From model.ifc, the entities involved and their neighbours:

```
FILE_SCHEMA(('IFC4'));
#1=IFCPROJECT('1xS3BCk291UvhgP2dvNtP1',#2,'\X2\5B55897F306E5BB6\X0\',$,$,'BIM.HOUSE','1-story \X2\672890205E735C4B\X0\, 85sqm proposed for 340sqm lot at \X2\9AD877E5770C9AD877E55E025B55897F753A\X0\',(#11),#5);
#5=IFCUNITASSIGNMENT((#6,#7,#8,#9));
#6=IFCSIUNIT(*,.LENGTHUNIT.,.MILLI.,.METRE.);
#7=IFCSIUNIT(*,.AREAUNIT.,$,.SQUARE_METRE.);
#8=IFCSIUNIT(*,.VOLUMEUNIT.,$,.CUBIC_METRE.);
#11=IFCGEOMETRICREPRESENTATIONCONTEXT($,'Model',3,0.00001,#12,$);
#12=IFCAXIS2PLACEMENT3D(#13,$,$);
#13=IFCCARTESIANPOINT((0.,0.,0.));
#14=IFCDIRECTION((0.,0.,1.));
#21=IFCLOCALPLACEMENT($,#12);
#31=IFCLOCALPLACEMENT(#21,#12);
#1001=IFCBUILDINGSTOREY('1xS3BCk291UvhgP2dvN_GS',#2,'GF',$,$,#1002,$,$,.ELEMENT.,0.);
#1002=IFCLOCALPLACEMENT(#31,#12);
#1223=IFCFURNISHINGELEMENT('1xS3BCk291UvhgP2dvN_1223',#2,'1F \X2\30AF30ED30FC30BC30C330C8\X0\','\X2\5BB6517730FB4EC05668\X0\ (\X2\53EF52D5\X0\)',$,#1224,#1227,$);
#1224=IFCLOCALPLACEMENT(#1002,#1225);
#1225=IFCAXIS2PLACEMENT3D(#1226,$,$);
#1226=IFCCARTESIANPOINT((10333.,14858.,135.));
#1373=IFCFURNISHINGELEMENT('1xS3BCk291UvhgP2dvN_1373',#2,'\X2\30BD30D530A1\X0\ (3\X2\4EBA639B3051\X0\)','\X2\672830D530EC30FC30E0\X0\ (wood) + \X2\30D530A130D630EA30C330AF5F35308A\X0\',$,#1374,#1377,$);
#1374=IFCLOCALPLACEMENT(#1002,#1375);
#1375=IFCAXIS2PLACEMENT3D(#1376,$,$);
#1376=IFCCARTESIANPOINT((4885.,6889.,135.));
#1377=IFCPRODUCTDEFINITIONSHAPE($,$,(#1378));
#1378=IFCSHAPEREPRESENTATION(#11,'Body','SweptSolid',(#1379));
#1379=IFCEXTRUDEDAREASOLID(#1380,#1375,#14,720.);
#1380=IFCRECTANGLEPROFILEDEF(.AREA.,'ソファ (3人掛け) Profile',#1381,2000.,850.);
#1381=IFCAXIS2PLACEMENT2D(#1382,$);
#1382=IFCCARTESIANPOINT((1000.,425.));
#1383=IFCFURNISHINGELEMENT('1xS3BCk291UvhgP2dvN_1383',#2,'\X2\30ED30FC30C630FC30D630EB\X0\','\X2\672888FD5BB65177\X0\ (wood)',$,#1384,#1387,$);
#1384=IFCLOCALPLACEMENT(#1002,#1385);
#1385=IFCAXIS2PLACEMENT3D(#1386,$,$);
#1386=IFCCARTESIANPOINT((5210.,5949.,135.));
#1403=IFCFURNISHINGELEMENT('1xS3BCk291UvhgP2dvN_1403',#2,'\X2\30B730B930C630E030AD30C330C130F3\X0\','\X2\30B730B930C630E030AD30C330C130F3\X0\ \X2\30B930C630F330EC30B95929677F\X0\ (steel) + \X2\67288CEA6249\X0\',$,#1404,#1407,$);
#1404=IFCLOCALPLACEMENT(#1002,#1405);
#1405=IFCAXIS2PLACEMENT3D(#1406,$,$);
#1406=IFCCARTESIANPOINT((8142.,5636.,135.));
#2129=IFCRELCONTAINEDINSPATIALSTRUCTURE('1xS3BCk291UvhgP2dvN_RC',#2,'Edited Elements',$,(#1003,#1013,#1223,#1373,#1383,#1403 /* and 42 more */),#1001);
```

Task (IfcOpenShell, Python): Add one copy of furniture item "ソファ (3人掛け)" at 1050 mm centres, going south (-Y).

```python
import numpy as np
import ifcopenshell
import ifcopenshell.api.geometry
import ifcopenshell.api.root
import ifcopenshell.util.element
import ifcopenshell.util.placement

model = ifcopenshell.open("model.ifc")


def reuse_history(source, copy):
    """copy_class also copies each property set's owner history, people and application; keep the originals."""
    for rel in copy.IsDefinedBy:
        if rel.is_a("IfcRelDefinesByProperties") and (history := rel.RelatingPropertyDefinition.OwnerHistory):
            rel.RelatingPropertyDefinition.OwnerHistory = source.OwnerHistory
            ifcopenshell.util.element.remove_deep2(model, history)


source = model.by_guid("1xS3BCk291UvhgP2dvN_1373")
base = ifcopenshell.util.placement.get_local_placement(source.ObjectPlacement)
step = np.array([0.0, -1.0, 0.0]) * 1050.0

for i in range(1, 2):
    copy = ifcopenshell.api.root.copy_class(model, product=source)
    copy.Representation = ifcopenshell.util.element.copy_deep(
        model, source.Representation, exclude=["IfcGeometricRepresentationContext", "IfcRepresentationMap"]
    )
    reuse_history(source, copy)
    matrix = base.copy()
    matrix[:3, 3] += i * step
    print("added at", matrix[:3, 3].round(3) + 0.0)
    ifcopenshell.api.geometry.edit_object_placement(model, product=copy, matrix=matrix, is_si=False)

model.write("model_rev.ifc")
```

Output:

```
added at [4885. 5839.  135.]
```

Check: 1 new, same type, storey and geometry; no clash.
